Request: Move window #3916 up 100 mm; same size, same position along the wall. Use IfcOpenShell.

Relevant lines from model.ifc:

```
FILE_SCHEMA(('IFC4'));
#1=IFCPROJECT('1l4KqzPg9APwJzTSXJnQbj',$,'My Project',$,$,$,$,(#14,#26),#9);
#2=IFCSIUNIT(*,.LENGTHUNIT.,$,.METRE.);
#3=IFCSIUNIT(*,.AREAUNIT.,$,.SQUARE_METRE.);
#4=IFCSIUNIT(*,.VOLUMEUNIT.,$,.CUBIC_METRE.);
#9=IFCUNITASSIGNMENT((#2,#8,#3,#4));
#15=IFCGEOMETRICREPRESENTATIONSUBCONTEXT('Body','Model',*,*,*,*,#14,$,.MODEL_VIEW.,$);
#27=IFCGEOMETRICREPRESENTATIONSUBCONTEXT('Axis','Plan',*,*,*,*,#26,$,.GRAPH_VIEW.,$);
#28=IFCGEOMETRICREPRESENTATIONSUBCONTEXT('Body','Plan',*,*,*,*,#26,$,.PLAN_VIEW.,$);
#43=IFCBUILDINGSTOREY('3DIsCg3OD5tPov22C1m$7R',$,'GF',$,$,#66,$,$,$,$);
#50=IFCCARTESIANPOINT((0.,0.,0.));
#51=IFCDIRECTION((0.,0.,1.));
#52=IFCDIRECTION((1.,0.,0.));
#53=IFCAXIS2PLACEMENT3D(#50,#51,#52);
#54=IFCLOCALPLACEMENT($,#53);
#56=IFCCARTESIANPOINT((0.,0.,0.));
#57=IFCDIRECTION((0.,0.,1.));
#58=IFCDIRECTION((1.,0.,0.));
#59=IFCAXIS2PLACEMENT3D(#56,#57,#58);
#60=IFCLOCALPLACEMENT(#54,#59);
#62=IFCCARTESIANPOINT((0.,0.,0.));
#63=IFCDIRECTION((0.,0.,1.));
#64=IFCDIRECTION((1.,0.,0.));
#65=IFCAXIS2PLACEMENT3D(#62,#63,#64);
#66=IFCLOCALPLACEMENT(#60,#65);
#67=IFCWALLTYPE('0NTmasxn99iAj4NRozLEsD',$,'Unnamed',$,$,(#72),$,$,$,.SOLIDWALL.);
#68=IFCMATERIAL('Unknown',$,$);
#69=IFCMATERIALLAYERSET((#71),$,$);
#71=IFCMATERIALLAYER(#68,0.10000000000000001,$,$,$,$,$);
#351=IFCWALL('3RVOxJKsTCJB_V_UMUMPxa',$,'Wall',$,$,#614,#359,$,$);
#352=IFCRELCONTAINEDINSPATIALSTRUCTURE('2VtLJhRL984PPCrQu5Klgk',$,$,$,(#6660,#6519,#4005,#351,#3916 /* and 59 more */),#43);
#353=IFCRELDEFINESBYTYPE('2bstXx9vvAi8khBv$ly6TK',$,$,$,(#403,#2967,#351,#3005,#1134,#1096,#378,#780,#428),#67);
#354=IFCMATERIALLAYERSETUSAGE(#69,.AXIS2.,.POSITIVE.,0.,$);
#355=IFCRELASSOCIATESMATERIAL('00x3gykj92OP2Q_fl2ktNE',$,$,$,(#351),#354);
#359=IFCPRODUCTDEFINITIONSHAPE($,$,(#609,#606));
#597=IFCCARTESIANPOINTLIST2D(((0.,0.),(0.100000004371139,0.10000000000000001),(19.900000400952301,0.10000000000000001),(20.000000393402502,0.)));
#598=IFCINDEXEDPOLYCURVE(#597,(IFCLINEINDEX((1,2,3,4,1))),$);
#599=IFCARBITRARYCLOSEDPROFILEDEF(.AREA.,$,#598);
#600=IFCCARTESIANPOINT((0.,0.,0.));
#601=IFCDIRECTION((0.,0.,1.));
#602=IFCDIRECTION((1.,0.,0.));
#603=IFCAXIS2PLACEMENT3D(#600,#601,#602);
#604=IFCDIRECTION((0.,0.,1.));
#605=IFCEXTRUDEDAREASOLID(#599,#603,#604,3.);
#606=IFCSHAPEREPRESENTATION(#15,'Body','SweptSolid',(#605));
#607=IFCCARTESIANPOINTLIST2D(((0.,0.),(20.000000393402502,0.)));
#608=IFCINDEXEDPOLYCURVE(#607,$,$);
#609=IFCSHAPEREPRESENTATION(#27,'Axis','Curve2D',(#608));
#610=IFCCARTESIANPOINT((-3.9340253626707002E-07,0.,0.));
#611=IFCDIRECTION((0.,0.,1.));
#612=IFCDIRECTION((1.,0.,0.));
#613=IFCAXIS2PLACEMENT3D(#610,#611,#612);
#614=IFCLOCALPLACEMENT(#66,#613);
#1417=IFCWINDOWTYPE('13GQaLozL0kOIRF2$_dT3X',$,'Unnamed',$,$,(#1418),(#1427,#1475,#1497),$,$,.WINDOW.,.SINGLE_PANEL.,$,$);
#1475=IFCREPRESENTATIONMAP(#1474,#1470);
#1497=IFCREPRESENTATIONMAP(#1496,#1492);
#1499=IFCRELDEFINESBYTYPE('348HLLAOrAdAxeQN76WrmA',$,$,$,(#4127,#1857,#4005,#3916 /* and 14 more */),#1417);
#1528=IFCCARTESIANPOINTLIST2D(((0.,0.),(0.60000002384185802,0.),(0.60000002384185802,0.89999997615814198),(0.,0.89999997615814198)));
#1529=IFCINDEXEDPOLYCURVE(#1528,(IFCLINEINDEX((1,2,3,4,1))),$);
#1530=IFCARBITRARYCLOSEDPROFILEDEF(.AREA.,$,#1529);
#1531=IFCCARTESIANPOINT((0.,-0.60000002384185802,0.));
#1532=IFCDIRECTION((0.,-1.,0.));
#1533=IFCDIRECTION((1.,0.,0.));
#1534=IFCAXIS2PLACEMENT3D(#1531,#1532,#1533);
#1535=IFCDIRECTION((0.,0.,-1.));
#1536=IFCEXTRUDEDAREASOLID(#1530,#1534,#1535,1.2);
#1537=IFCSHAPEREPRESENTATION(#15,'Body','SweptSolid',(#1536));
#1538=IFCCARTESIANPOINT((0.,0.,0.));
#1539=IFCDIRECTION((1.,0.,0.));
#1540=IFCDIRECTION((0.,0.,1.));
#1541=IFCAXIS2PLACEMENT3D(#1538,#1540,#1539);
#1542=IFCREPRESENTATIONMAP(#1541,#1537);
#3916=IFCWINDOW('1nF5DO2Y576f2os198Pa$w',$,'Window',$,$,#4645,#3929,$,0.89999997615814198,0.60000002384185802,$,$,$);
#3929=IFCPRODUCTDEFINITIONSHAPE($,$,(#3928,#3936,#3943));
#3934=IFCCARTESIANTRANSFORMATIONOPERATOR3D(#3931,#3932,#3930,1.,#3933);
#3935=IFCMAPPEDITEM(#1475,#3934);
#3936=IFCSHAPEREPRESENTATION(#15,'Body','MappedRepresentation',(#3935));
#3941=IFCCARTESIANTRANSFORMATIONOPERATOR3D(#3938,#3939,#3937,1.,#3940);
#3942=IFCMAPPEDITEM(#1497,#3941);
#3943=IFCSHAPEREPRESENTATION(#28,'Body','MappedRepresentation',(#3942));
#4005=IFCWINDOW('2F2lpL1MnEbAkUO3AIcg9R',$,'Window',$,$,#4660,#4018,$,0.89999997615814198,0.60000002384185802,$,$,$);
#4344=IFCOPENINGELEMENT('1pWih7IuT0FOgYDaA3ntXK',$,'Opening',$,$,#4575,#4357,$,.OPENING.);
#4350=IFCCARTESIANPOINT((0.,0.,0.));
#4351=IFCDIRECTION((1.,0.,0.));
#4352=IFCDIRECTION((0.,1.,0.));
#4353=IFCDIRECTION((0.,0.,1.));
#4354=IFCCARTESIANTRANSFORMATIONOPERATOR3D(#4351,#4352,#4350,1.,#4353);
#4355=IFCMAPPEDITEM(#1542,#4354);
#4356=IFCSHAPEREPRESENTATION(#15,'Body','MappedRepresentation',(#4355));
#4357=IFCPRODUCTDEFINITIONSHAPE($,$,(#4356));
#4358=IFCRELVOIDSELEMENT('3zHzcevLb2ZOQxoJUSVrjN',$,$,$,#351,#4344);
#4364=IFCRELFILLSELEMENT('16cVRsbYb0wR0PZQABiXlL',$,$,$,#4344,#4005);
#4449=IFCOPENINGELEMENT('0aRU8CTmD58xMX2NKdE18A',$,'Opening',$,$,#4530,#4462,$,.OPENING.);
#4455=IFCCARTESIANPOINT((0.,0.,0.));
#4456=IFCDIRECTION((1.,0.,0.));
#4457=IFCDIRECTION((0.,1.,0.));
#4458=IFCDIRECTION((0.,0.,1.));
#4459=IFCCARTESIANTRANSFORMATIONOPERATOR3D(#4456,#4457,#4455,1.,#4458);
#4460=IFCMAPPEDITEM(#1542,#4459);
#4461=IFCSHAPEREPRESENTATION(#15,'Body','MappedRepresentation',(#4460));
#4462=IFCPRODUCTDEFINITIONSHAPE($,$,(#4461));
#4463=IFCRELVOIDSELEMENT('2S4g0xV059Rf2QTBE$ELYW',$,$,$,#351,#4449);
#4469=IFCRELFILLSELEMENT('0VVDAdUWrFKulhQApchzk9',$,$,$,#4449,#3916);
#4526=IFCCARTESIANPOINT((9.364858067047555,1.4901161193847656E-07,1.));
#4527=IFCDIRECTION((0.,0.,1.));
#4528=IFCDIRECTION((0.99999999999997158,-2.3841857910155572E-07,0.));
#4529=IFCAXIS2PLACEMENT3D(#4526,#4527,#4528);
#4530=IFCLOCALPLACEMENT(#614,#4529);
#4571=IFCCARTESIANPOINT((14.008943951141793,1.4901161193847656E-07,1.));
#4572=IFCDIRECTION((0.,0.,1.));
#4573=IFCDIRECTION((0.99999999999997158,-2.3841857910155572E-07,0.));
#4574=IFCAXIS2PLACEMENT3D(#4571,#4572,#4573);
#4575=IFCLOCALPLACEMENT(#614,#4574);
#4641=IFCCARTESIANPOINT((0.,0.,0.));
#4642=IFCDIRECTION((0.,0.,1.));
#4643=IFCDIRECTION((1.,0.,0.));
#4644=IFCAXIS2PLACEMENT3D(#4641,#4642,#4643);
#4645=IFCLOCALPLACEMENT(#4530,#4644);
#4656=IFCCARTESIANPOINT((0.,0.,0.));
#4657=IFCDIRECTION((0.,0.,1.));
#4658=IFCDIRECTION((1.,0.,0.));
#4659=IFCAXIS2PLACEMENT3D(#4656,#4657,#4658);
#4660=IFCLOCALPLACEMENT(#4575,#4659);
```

```python
import numpy as np
import ifcopenshell
import ifcopenshell.api.geometry
import ifcopenshell.util.placement
import ifcopenshell.util.unit

model = ifcopenshell.open("model.ifc")
unit_scale = ifcopenshell.util.unit.calculate_unit_scale(model)

window = model.by_guid("1nF5DO2Y576f2os198Pa$w")
opening = window.FillsVoids[0].RelatingOpeningElement
dz = 0.1

shift = np.array([0.0, 0.0, dz])
# The window is placed relative to its opening, so it follows when the opening moves.
matrix = ifcopenshell.util.placement.get_local_placement(opening.ObjectPlacement)
matrix[:3, 3] += shift
ifcopenshell.api.geometry.edit_object_placement(
    model, product=opening, matrix=matrix, is_si=False, should_transform_children=True
)

print(f"moved by {dz * unit_scale:+.3f} m")

model.write("model-out.ifc")
```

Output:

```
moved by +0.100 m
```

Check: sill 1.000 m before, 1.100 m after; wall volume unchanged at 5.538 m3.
